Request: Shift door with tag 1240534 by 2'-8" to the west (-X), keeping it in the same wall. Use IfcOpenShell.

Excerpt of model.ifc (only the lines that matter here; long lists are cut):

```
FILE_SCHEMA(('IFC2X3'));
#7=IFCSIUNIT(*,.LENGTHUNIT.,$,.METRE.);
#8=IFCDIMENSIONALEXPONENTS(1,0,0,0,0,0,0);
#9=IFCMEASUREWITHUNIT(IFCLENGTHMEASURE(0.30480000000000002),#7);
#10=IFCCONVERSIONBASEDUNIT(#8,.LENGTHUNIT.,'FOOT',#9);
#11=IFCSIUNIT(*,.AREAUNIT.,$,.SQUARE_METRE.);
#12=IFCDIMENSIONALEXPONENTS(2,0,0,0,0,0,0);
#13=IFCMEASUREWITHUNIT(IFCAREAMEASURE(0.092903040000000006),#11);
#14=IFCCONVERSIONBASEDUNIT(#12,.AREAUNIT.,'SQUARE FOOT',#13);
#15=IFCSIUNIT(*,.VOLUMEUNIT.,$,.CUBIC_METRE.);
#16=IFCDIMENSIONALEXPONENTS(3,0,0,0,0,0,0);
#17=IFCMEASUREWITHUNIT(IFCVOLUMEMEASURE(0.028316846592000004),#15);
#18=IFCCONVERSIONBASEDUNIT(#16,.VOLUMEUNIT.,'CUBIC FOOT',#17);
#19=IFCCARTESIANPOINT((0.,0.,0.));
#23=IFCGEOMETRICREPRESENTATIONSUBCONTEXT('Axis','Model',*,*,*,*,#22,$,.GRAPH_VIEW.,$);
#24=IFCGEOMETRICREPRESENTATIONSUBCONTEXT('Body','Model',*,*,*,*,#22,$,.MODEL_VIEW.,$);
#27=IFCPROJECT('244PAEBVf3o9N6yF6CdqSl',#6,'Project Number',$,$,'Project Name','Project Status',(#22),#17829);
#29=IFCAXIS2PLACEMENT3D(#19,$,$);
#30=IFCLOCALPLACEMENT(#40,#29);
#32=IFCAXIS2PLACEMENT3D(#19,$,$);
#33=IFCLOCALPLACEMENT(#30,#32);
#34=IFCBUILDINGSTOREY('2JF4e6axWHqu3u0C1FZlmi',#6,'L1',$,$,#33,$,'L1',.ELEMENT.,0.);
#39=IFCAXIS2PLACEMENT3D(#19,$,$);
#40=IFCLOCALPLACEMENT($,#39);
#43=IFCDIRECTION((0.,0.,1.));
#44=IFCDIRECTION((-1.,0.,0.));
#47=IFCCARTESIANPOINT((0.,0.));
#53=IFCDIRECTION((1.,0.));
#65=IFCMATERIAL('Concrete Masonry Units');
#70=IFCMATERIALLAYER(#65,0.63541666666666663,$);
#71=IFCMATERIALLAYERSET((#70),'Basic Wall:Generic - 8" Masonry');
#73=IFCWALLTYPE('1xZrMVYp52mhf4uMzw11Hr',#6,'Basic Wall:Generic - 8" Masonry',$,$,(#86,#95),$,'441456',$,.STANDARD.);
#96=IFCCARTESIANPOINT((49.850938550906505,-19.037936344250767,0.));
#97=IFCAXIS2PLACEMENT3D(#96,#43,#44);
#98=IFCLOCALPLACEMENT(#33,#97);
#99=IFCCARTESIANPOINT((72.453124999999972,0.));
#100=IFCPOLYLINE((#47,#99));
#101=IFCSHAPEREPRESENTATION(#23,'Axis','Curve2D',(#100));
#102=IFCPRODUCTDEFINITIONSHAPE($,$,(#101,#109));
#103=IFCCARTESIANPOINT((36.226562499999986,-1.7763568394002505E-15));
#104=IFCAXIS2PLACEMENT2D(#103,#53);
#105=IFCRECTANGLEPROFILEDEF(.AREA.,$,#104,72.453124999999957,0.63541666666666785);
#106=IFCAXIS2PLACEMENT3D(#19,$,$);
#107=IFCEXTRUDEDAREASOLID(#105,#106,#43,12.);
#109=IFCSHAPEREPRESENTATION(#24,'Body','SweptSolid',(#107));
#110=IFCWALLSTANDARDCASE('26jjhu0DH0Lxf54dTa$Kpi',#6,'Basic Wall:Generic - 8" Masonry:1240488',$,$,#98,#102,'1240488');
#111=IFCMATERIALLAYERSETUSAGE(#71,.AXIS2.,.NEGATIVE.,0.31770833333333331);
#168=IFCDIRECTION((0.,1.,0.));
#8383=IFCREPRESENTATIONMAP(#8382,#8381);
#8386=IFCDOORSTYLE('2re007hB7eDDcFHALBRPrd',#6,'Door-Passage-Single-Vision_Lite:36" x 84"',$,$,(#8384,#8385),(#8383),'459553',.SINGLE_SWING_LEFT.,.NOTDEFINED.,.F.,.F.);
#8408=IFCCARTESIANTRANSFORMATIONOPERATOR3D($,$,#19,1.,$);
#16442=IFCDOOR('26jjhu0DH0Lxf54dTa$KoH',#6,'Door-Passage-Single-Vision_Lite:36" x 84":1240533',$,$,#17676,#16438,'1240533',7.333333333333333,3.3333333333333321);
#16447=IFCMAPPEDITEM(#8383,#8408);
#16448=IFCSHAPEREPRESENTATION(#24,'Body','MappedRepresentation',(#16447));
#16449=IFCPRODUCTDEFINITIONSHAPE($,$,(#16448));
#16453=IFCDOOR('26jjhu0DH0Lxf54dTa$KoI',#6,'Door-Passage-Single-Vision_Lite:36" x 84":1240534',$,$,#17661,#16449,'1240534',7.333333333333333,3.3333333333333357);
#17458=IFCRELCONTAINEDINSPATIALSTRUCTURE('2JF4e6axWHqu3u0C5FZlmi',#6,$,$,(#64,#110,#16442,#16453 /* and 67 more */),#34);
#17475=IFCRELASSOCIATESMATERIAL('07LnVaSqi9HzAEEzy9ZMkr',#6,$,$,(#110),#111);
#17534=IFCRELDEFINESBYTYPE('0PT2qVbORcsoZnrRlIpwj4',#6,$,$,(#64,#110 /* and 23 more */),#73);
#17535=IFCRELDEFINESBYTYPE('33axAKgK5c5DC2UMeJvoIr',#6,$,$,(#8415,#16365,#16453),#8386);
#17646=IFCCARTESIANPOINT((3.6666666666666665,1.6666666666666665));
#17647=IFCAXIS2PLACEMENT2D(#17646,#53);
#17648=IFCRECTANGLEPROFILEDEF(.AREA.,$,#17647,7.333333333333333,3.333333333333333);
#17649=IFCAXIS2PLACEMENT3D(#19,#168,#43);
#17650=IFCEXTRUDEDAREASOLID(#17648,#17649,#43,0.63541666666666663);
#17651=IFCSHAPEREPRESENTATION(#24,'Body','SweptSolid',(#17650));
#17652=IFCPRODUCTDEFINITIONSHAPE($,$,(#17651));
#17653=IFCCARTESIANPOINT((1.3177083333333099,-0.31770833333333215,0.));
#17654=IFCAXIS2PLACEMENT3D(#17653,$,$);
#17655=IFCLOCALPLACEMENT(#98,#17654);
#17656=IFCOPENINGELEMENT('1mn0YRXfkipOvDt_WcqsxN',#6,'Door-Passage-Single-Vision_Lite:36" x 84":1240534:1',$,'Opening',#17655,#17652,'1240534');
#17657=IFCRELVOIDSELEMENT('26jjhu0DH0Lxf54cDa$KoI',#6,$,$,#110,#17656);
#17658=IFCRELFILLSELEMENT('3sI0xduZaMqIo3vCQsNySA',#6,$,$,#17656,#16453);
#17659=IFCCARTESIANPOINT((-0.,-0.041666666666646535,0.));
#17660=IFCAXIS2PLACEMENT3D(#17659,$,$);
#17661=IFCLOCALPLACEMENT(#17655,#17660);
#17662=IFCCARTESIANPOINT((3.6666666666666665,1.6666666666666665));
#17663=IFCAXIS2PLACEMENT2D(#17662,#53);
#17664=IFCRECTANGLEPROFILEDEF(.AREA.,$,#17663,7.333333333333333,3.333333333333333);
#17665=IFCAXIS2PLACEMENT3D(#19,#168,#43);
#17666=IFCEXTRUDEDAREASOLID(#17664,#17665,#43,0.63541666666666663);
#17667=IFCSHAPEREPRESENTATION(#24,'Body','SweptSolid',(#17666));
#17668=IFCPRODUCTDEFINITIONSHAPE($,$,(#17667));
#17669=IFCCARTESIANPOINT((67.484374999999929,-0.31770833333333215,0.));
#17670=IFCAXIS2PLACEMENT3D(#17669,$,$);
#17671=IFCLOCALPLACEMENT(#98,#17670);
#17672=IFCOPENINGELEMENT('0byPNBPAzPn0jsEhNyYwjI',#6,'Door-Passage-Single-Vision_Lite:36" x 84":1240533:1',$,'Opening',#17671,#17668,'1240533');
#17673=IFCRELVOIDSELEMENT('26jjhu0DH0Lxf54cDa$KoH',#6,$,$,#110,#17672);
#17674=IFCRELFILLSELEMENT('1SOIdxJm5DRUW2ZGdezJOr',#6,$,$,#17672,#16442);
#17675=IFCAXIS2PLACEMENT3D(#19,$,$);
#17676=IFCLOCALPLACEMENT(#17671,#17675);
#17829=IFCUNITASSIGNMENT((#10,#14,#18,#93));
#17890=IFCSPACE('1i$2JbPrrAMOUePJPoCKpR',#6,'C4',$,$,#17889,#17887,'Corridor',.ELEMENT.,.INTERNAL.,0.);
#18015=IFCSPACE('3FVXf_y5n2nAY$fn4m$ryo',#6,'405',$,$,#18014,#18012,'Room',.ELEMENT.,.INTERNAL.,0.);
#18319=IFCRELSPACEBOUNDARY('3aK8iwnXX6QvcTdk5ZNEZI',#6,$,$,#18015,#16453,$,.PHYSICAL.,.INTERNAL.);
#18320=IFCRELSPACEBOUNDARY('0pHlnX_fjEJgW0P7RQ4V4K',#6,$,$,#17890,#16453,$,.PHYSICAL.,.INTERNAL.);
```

```python
import ifcopenshell
import ifcopenshell.api.geometry
import ifcopenshell.util.placement
import ifcopenshell.util.unit

model = ifcopenshell.open("model.ifc")
unit_scale = ifcopenshell.util.unit.calculate_unit_scale(model)

door = model.by_guid("26jjhu0DH0Lxf54dTa$KoI")
opening = door.FillsVoids[0].RelatingOpeningElement
wall = opening.VoidsElements[0].RelatingBuildingElement

wall_matrix = ifcopenshell.util.placement.get_local_placement(wall.ObjectPlacement)
shift = wall_matrix[:3, 0] * 32 * 0.0254 / unit_scale
before = ifcopenshell.util.placement.get_local_placement(door.ObjectPlacement)[:3, 3].copy()

# The door is placed relative to its opening, so it follows when the opening moves.
matrix = ifcopenshell.util.placement.get_local_placement(opening.ObjectPlacement)
matrix[:3, 3] += shift
ifcopenshell.api.geometry.edit_object_placement(
    model, product=opening, matrix=matrix, is_si=False, should_transform_children=True
)

after = ifcopenshell.util.placement.get_local_placement(door.ObjectPlacement)[:3, 3]
print("door moved by", (after - before).round(3) + 0.0)

model.write("model_updated.ifc")
```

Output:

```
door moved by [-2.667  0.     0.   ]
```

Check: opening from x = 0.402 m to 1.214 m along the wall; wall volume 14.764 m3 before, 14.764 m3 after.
